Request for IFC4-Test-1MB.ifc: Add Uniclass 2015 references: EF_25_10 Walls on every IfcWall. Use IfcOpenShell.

First a look at what the model holds.

```python
import ifcopenshell

model = ifcopenshell.open("IFC4-Test-1MB.ifc")
print(model.schema)
print("classifications:", [c.Name for c in model.by_type("IfcClassification")])
for ifc_class in ("IfcDoor", "IfcRoof", "IfcStair", "IfcWall", "IfcWindow"):
    print(ifc_class, len(model.by_type(ifc_class)))
```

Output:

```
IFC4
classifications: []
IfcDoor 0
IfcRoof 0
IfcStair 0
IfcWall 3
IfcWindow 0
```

```python
import ifcopenshell
import ifcopenshell.api.classification

model = ifcopenshell.open("IFC4-Test-1MB.ifc")

system = ifcopenshell.api.classification.add_classification(model, classification="Uniclass 2015")

codes = {
    "IfcWall": ("EF_25_10", "Walls"),
}
for ifc_class, (code, name) in codes.items():
    products = model.by_type(ifc_class)
    ifcopenshell.api.classification.add_reference(
        model, products=products, classification=system, identification=code, name=name
    )
    print(code, len(products))

model.write("IFC4-Test-1MB_rev.ifc")
```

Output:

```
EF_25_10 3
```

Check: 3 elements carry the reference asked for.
